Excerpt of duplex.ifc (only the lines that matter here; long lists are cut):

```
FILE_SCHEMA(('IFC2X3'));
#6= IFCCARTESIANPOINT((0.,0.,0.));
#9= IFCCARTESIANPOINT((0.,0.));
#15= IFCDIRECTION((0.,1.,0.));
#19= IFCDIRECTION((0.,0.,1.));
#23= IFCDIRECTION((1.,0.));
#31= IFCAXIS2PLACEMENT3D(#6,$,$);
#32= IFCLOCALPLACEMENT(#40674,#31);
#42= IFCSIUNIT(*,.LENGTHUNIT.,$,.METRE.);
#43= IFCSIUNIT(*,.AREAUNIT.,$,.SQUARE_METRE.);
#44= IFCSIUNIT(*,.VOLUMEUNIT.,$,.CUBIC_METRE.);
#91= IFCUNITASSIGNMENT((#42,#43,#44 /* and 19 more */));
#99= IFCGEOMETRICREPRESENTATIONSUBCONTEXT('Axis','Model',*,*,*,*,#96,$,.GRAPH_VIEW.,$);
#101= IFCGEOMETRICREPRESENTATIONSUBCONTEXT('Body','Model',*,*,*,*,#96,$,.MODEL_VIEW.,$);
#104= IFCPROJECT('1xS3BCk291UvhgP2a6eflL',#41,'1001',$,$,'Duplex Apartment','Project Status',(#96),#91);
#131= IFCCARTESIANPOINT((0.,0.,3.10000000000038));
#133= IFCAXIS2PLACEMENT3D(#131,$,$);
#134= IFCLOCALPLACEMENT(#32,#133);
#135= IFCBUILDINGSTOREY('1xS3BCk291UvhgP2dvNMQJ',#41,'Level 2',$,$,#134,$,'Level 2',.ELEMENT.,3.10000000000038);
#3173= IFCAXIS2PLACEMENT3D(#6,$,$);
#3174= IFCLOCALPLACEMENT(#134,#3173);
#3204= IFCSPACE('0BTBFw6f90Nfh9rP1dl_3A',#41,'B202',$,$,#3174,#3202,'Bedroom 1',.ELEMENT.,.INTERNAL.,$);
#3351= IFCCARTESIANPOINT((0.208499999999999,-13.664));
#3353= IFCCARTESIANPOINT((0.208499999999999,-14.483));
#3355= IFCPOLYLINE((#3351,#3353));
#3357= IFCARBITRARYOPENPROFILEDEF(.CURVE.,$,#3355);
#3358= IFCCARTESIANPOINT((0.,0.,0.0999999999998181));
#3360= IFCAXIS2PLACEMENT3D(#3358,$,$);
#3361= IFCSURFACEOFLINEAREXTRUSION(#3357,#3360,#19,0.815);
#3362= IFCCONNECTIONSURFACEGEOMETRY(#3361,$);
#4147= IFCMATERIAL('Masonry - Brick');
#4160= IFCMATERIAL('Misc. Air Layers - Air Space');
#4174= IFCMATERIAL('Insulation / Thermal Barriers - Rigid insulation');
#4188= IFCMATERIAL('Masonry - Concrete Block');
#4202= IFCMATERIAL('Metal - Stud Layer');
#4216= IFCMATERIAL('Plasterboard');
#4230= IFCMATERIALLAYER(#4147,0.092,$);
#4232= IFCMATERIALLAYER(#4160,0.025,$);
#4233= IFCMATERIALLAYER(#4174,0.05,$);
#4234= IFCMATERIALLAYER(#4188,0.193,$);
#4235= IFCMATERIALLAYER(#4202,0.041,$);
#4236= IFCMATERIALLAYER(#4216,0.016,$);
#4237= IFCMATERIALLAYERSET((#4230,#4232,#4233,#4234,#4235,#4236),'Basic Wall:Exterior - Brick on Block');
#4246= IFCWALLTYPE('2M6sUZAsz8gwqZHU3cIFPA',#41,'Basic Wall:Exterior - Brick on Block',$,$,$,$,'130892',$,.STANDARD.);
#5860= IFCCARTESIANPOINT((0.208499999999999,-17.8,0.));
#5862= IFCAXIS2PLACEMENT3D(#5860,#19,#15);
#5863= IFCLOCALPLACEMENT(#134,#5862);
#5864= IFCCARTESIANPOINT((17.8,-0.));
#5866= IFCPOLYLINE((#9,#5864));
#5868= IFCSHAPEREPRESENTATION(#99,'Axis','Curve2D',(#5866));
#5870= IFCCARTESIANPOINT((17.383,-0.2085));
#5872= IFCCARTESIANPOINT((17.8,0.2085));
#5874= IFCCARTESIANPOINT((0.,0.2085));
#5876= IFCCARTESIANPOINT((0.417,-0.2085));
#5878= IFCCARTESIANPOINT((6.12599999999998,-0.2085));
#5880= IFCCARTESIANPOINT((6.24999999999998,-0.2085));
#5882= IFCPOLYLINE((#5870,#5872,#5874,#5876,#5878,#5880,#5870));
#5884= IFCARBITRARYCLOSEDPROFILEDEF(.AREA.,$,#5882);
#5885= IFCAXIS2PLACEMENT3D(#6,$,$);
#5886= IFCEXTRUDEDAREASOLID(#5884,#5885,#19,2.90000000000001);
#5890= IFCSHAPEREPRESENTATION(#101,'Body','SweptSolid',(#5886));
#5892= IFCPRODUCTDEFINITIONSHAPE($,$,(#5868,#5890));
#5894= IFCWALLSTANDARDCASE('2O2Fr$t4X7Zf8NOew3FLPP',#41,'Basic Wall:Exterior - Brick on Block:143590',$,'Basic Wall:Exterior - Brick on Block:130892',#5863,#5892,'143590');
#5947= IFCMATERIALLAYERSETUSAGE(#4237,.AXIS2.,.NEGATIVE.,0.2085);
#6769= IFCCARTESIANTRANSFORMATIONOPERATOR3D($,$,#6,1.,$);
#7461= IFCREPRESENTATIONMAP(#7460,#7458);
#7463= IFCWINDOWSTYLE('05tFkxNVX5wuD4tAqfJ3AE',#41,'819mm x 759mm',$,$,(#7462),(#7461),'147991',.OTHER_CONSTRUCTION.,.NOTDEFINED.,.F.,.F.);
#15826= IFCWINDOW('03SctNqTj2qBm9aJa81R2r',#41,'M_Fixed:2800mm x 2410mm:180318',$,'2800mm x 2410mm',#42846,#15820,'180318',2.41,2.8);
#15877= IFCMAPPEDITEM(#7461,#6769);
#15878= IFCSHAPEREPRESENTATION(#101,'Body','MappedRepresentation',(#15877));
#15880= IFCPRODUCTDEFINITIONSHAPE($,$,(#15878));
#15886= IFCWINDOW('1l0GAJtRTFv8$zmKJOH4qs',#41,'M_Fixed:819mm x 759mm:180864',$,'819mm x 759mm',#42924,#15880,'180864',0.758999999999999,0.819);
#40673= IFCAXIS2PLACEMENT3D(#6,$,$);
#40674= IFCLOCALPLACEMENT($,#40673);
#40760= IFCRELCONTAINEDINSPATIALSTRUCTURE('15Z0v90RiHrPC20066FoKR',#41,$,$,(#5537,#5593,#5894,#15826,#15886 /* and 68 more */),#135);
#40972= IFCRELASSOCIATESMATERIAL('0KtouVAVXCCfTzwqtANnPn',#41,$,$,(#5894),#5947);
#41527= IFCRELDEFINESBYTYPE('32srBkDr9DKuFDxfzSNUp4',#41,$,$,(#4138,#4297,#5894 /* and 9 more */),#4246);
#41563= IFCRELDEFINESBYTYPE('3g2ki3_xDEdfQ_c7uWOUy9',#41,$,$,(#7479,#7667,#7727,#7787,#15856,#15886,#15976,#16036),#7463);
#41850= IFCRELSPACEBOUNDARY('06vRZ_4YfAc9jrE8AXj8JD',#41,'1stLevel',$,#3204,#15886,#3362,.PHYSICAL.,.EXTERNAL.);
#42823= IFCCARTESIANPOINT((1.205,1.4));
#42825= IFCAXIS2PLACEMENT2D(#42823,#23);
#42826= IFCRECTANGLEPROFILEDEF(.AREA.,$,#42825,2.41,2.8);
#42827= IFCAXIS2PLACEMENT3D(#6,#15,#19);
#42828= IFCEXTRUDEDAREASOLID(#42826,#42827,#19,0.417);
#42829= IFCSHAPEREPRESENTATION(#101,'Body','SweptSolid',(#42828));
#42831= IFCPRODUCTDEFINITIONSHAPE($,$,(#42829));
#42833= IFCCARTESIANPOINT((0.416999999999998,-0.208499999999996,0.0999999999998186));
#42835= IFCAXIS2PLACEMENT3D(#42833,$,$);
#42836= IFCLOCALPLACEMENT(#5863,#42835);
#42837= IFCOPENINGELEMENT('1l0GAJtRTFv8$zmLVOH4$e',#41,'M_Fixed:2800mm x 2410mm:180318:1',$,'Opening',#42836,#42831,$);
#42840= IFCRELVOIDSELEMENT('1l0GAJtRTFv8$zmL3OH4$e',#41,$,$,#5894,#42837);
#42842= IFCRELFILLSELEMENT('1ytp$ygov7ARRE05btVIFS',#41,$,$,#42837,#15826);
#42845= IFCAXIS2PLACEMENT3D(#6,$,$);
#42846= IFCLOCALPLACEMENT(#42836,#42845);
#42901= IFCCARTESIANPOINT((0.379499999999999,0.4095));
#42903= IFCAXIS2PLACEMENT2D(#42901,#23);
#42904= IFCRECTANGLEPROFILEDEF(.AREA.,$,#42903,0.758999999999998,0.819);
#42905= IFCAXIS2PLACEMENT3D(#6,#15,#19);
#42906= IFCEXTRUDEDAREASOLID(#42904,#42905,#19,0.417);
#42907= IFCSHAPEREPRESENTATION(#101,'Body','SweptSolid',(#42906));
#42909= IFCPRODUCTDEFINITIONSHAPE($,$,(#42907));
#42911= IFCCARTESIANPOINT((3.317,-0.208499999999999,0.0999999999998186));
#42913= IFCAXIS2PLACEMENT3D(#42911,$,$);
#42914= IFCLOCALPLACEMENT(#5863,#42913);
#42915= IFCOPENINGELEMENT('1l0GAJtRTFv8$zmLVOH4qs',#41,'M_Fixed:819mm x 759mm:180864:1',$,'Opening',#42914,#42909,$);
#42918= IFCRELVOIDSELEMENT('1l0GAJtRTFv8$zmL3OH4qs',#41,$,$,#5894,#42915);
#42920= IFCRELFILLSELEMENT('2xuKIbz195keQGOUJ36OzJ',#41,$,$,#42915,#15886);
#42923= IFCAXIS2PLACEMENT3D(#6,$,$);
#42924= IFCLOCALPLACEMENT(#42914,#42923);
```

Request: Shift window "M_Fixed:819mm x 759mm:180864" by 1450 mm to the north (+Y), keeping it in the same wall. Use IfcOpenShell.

```python
import numpy as np
import ifcopenshell
import ifcopenshell.api.geometry
import ifcopenshell.util.placement

model = ifcopenshell.open("duplex.ifc")

window = model.by_guid("1l0GAJtRTFv8$zmKJOH4qs")
opening = window.FillsVoids[0].RelatingOpeningElement
wall = opening.VoidsElements[0].RelatingBuildingElement

wall_matrix = ifcopenshell.util.placement.get_local_placement(wall.ObjectPlacement)
shift = wall_matrix[:3, 0] * 1.45
before = ifcopenshell.util.placement.get_local_placement(window.ObjectPlacement)[:3, 3].copy()

# The window is placed relative to its opening, so it follows when the opening moves.
matrix = ifcopenshell.util.placement.get_local_placement(opening.ObjectPlacement)
matrix[:3, 3] += shift
ifcopenshell.api.geometry.edit_object_placement(
    model, product=opening, matrix=matrix, is_si=False, should_transform_children=True
)

# Space boundary surfaces are stored in each space's coordinates; move them too.
for rel in window.ProvidesBoundaries:
    if not rel.ConnectionGeometry:
        continue
    surface = rel.ConnectionGeometry.SurfaceOnRelatingElement
    space_matrix = ifcopenshell.util.placement.get_local_placement(rel.RelatingSpace.ObjectPlacement)
    point = np.array(surface.Position.Location.Coordinates) + space_matrix[:3, :3].T @ shift
    surface.Position = model.createIfcAxis2Placement3D(
        model.createIfcCartesianPoint(point.tolist()), surface.Position.Axis, surface.Position.RefDirection
    )

after = ifcopenshell.util.placement.get_local_placement(window.ObjectPlacement)[:3, 3]
print("window moved by", (after - before).round(3) + 0.0)

model.write("duplex_v2.ifc")
```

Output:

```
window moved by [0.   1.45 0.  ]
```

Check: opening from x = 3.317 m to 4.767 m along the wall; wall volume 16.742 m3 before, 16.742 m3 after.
